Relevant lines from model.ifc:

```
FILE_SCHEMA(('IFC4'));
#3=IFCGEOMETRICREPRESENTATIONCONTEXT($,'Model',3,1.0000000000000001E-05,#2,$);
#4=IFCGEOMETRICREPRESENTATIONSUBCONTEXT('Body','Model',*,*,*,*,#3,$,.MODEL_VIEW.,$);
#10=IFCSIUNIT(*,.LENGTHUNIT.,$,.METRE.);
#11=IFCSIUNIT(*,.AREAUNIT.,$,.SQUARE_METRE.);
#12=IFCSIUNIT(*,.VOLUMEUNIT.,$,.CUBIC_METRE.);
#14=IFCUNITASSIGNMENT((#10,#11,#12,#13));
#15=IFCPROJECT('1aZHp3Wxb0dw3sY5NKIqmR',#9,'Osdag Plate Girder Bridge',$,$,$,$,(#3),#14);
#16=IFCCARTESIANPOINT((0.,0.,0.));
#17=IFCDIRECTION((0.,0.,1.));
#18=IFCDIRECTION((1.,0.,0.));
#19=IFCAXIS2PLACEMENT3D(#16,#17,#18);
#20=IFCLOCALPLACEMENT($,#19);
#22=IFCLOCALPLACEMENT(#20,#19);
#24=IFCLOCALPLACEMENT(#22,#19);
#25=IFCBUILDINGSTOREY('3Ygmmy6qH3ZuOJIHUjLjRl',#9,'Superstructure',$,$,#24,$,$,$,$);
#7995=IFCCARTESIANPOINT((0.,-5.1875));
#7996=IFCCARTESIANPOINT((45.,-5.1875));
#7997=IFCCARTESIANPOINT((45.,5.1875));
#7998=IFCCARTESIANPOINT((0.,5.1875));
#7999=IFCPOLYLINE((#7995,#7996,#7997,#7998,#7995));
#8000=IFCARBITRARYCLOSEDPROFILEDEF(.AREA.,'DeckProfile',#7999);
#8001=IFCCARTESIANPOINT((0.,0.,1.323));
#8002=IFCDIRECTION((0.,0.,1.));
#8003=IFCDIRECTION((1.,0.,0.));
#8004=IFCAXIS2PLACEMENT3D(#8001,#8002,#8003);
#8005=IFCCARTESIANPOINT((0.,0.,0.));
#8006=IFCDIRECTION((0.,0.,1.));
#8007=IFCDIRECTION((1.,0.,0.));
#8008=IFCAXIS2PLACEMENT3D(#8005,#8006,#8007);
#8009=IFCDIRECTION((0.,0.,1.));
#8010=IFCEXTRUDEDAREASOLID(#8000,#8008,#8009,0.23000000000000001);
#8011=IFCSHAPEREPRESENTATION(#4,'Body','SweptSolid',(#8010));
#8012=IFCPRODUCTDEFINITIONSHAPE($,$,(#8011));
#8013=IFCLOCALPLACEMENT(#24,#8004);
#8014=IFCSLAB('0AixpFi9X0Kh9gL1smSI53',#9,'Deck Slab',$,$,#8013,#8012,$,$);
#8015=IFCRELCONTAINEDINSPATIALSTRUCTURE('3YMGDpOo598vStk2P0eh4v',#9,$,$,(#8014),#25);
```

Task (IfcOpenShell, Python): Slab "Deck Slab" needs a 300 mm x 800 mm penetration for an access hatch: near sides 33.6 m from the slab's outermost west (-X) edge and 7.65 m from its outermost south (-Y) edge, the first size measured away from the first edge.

```python
import numpy as np
import ifcopenshell
import ifcopenshell.api.feature
import ifcopenshell.api.geometry
import ifcopenshell.api.root
import ifcopenshell.geom
import ifcopenshell.util.placement
import ifcopenshell.util.representation
import ifcopenshell.util.shape
import ifcopenshell.util.unit

model = ifcopenshell.open("model.ifc")
unit_scale = ifcopenshell.util.unit.calculate_unit_scale(model)
settings = ifcopenshell.geom.settings()


def volume(element):
    """Net volume in cubic metres, openings subtracted."""
    shape = ifcopenshell.geom.create_shape(settings, element)
    return ifcopenshell.util.shape.get_volume(shape.geometry)


slab = model.by_guid("0AixpFi9X0Kh9gL1smSI53")
before = volume(slab)

# Extent in the slab's own axes, in metres. The edges named are its -X and -Y sides.
slab_shape = ifcopenshell.geom.create_shape(settings, slab)
vertices = ifcopenshell.util.shape.get_vertices(slab_shape.geometry)
x_min, y_min, bottom = vertices.min(axis=0)
top = vertices[:, 2].max()

opening = ifcopenshell.api.root.create_entity(model, ifc_class="IfcOpeningElement", name="Access hatch opening", predefined_type="OPENING")
context = ifcopenshell.util.representation.get_context(model, "Model", "Body", "MODEL_VIEW")
width, depth = 0.3, 0.8
outline = [(0.0, 0.0), (width, 0.0), (width, depth), (0.0, depth), (0.0, 0.0)]
# Overshoot both faces by 50 mm so the cut is clean.
shape = ifcopenshell.api.geometry.add_slab_representation(
    model, context=context, depth=top - bottom + 0.1, polyline=outline
)
ifcopenshell.api.geometry.assign_representation(model, product=opening, representation=shape)

matrix = ifcopenshell.util.placement.get_local_placement(slab.ObjectPlacement)
matrix[:, 3] = matrix @ np.append(np.array([x_min + 33.6, y_min + 7.65, bottom - 0.05]) / unit_scale, 1.0)
ifcopenshell.api.geometry.edit_object_placement(model, product=opening, matrix=matrix, is_si=False)
ifcopenshell.api.feature.add_feature(model, feature=opening, element=slab)

after = volume(slab)

print(f"slab volume {before:.3f} -> {after:.3f} m3")

model.write("model_edited.ifc")
```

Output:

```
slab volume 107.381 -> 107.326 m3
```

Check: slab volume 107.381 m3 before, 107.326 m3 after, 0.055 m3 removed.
